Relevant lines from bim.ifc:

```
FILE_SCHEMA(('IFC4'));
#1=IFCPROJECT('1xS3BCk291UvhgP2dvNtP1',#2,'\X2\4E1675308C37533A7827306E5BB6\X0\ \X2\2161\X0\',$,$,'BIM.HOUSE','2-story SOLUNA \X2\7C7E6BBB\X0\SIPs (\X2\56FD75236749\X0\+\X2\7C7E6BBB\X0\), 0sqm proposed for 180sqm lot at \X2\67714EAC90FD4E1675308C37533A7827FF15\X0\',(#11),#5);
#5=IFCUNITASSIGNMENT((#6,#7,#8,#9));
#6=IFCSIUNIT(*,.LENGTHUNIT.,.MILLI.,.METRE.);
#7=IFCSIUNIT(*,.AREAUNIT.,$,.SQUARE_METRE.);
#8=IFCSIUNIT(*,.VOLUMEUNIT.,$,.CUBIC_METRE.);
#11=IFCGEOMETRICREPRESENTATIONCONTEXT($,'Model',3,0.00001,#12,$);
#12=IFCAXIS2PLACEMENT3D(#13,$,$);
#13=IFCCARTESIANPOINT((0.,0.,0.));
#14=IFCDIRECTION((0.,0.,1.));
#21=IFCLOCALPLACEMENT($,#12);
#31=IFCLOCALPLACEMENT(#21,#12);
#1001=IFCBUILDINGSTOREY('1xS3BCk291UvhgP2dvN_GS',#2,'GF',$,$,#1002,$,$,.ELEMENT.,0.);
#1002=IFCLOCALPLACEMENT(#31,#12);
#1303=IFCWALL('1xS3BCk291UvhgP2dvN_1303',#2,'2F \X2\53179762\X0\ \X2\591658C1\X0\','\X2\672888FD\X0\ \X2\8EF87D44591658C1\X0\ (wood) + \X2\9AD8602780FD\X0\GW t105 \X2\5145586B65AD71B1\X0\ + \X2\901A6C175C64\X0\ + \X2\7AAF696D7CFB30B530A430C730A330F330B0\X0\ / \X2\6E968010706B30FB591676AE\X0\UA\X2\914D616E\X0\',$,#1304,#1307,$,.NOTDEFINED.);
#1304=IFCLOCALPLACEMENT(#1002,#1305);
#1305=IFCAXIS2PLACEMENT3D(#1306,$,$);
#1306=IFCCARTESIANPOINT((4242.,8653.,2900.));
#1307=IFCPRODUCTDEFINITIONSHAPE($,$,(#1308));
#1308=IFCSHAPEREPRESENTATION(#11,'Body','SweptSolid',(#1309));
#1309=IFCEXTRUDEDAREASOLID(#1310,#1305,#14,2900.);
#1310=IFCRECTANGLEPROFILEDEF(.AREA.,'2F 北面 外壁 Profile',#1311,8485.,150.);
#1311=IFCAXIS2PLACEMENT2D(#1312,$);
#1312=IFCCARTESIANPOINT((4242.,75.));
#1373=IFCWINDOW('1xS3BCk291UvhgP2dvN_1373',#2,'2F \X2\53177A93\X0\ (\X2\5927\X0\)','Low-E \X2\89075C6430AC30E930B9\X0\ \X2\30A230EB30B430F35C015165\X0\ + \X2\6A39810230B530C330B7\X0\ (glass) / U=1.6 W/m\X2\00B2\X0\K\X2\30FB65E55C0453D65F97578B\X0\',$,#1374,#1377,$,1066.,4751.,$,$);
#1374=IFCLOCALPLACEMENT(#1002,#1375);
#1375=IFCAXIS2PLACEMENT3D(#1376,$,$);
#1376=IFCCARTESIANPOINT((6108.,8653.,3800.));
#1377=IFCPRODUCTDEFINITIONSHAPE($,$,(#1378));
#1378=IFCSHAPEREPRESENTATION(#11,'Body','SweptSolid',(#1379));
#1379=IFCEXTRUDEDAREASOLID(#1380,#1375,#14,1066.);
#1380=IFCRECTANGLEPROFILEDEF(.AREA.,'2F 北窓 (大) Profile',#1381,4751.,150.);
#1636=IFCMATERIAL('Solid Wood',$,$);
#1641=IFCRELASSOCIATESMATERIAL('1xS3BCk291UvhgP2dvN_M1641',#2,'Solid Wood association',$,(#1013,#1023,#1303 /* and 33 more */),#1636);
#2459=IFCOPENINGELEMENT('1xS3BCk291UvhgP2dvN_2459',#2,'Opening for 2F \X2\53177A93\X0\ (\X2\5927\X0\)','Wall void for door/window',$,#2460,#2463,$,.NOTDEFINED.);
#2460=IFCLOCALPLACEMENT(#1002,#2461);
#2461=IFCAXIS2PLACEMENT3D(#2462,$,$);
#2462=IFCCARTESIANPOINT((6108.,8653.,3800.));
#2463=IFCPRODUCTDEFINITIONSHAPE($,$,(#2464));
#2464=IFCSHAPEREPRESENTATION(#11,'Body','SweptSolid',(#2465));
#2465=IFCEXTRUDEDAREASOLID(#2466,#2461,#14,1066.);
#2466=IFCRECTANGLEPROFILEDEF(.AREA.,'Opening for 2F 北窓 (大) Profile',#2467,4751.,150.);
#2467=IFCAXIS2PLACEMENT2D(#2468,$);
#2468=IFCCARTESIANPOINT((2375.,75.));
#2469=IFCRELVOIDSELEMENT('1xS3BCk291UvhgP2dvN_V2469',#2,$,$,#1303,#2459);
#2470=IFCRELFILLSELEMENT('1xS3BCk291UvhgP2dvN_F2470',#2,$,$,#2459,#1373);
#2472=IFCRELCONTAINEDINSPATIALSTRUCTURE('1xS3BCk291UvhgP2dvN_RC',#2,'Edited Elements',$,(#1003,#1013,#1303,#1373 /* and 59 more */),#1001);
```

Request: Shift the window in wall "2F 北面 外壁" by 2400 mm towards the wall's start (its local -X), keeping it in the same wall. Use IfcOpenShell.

```python
import ifcopenshell
import ifcopenshell.api.geometry
import ifcopenshell.util.placement

model = ifcopenshell.open("bim.ifc")

window = model.by_id(1373)
opening = window.FillsVoids[0].RelatingOpeningElement
wall = opening.VoidsElements[0].RelatingBuildingElement

wall_matrix = ifcopenshell.util.placement.get_local_placement(wall.ObjectPlacement)
shift = wall_matrix[:3, 0] * -2400.0
before = ifcopenshell.util.placement.get_local_placement(window.ObjectPlacement)[:3, 3].copy()

# The window is not placed relative to its opening, so move both.
for product in (opening, window):
    matrix = ifcopenshell.util.placement.get_local_placement(product.ObjectPlacement)
    matrix[:3, 3] += shift
    ifcopenshell.api.geometry.edit_object_placement(model, product=product, matrix=matrix, is_si=False)

after = ifcopenshell.util.placement.get_local_placement(window.ObjectPlacement)[:3, 3]
print("window moved by", (after - before).round(3) + 0.0)

model.write("bim_edited.ifc")
```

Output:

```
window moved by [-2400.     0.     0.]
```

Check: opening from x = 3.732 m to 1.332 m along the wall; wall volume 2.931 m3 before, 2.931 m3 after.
